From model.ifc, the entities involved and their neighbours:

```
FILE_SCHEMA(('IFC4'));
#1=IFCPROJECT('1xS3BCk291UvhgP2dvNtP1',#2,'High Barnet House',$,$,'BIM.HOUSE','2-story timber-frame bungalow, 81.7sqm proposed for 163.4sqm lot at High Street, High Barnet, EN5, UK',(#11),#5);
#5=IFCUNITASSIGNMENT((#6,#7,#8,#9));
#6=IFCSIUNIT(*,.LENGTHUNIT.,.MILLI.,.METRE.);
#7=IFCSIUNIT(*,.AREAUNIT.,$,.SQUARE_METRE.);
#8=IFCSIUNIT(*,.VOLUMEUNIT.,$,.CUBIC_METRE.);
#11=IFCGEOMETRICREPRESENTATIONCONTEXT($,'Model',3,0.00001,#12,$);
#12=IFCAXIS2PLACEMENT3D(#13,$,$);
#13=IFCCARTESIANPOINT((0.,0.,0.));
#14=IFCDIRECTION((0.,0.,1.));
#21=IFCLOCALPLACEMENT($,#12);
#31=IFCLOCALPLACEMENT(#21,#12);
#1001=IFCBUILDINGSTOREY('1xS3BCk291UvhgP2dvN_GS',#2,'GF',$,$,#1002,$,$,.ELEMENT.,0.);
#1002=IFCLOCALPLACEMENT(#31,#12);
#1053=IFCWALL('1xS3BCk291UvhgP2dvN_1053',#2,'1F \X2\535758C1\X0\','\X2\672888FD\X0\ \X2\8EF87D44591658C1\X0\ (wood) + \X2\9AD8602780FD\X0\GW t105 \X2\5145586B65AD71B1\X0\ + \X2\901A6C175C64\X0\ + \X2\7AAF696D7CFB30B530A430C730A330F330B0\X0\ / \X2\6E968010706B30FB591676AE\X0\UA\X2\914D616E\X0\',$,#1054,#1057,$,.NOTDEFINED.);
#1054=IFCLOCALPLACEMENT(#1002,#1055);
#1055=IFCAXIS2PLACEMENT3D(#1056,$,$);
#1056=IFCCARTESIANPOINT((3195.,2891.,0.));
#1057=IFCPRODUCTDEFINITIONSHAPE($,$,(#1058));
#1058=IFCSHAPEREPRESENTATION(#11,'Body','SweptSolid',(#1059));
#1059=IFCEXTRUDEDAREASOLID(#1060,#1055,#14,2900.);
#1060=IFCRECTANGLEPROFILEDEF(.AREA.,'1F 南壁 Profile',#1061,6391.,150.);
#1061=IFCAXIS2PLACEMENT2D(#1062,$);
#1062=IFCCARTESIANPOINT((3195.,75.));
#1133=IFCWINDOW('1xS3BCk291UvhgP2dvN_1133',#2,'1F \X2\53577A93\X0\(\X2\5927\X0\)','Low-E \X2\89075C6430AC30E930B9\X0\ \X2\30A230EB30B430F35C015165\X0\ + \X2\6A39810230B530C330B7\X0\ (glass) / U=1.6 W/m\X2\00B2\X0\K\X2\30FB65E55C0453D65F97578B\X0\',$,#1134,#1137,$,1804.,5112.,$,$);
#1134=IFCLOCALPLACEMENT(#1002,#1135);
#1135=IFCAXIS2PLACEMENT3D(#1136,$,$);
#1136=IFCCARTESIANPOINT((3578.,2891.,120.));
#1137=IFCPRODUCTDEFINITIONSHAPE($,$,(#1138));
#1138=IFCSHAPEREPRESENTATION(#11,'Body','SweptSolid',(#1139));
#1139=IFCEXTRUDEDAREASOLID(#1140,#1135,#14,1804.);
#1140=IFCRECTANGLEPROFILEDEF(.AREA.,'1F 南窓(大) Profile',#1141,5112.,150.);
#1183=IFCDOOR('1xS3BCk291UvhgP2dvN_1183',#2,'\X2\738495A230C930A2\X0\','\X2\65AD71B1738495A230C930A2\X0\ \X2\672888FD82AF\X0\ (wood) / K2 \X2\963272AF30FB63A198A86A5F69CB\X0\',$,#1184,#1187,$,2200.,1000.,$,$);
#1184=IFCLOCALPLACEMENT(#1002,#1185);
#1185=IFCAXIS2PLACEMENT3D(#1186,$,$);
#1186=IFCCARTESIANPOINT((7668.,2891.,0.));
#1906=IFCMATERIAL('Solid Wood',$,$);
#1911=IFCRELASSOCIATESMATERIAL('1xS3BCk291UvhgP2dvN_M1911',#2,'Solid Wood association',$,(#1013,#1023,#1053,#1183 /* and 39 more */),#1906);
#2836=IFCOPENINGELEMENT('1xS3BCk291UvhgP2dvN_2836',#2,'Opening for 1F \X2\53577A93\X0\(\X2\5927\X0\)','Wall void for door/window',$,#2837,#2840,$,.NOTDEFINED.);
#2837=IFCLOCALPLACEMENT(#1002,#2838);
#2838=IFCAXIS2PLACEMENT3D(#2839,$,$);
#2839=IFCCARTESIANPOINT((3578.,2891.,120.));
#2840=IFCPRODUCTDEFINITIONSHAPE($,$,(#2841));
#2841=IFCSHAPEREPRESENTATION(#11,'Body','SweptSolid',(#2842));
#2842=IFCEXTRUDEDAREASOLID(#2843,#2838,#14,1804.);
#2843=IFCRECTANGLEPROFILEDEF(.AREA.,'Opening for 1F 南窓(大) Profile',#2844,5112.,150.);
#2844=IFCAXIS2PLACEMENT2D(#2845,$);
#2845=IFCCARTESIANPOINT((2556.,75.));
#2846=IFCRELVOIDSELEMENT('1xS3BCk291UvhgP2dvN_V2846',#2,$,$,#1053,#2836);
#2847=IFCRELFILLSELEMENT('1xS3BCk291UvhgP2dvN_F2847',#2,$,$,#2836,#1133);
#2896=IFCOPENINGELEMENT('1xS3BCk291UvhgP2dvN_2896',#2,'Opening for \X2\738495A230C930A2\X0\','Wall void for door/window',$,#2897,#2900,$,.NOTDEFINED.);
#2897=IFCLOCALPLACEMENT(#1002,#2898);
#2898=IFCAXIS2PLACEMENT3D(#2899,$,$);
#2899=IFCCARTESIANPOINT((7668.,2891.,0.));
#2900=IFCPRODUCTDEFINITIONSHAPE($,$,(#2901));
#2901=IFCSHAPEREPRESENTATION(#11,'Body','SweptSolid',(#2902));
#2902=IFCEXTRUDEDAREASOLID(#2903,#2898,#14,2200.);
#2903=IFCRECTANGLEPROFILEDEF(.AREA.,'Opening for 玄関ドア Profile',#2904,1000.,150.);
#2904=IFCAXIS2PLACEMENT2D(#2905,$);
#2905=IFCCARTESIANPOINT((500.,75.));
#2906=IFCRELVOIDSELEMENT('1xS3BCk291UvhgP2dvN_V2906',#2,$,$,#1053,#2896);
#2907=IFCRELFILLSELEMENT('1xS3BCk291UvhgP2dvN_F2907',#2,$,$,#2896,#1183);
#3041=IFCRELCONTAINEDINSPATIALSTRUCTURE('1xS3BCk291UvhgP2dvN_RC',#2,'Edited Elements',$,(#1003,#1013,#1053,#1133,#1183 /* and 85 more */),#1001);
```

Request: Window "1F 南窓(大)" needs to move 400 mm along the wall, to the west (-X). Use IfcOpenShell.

```python
import ifcopenshell
import ifcopenshell.api.geometry
import ifcopenshell.util.placement
import ifcopenshell.util.unit

model = ifcopenshell.open("model.ifc")
unit_scale = ifcopenshell.util.unit.calculate_unit_scale(model)

window = model.by_id(1133)
opening = window.FillsVoids[0].RelatingOpeningElement
wall = opening.VoidsElements[0].RelatingBuildingElement

wall_matrix = ifcopenshell.util.placement.get_local_placement(wall.ObjectPlacement)
shift = wall_matrix[:3, 0] * -0.4 / unit_scale
before = ifcopenshell.util.placement.get_local_placement(window.ObjectPlacement)[:3, 3].copy()

# The window is not placed relative to its opening, so move both.
for product in (opening, window):
    matrix = ifcopenshell.util.placement.get_local_placement(product.ObjectPlacement)
    matrix[:3, 3] += shift
    ifcopenshell.api.geometry.edit_object_placement(model, product=product, matrix=matrix, is_si=False)

after = ifcopenshell.util.placement.get_local_placement(window.ObjectPlacement)[:3, 3]
print("window moved by", (after - before).round(3) + 0.0)

model.write("model_updated.ifc")
```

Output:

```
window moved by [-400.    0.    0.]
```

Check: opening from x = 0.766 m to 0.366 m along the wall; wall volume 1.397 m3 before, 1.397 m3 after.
